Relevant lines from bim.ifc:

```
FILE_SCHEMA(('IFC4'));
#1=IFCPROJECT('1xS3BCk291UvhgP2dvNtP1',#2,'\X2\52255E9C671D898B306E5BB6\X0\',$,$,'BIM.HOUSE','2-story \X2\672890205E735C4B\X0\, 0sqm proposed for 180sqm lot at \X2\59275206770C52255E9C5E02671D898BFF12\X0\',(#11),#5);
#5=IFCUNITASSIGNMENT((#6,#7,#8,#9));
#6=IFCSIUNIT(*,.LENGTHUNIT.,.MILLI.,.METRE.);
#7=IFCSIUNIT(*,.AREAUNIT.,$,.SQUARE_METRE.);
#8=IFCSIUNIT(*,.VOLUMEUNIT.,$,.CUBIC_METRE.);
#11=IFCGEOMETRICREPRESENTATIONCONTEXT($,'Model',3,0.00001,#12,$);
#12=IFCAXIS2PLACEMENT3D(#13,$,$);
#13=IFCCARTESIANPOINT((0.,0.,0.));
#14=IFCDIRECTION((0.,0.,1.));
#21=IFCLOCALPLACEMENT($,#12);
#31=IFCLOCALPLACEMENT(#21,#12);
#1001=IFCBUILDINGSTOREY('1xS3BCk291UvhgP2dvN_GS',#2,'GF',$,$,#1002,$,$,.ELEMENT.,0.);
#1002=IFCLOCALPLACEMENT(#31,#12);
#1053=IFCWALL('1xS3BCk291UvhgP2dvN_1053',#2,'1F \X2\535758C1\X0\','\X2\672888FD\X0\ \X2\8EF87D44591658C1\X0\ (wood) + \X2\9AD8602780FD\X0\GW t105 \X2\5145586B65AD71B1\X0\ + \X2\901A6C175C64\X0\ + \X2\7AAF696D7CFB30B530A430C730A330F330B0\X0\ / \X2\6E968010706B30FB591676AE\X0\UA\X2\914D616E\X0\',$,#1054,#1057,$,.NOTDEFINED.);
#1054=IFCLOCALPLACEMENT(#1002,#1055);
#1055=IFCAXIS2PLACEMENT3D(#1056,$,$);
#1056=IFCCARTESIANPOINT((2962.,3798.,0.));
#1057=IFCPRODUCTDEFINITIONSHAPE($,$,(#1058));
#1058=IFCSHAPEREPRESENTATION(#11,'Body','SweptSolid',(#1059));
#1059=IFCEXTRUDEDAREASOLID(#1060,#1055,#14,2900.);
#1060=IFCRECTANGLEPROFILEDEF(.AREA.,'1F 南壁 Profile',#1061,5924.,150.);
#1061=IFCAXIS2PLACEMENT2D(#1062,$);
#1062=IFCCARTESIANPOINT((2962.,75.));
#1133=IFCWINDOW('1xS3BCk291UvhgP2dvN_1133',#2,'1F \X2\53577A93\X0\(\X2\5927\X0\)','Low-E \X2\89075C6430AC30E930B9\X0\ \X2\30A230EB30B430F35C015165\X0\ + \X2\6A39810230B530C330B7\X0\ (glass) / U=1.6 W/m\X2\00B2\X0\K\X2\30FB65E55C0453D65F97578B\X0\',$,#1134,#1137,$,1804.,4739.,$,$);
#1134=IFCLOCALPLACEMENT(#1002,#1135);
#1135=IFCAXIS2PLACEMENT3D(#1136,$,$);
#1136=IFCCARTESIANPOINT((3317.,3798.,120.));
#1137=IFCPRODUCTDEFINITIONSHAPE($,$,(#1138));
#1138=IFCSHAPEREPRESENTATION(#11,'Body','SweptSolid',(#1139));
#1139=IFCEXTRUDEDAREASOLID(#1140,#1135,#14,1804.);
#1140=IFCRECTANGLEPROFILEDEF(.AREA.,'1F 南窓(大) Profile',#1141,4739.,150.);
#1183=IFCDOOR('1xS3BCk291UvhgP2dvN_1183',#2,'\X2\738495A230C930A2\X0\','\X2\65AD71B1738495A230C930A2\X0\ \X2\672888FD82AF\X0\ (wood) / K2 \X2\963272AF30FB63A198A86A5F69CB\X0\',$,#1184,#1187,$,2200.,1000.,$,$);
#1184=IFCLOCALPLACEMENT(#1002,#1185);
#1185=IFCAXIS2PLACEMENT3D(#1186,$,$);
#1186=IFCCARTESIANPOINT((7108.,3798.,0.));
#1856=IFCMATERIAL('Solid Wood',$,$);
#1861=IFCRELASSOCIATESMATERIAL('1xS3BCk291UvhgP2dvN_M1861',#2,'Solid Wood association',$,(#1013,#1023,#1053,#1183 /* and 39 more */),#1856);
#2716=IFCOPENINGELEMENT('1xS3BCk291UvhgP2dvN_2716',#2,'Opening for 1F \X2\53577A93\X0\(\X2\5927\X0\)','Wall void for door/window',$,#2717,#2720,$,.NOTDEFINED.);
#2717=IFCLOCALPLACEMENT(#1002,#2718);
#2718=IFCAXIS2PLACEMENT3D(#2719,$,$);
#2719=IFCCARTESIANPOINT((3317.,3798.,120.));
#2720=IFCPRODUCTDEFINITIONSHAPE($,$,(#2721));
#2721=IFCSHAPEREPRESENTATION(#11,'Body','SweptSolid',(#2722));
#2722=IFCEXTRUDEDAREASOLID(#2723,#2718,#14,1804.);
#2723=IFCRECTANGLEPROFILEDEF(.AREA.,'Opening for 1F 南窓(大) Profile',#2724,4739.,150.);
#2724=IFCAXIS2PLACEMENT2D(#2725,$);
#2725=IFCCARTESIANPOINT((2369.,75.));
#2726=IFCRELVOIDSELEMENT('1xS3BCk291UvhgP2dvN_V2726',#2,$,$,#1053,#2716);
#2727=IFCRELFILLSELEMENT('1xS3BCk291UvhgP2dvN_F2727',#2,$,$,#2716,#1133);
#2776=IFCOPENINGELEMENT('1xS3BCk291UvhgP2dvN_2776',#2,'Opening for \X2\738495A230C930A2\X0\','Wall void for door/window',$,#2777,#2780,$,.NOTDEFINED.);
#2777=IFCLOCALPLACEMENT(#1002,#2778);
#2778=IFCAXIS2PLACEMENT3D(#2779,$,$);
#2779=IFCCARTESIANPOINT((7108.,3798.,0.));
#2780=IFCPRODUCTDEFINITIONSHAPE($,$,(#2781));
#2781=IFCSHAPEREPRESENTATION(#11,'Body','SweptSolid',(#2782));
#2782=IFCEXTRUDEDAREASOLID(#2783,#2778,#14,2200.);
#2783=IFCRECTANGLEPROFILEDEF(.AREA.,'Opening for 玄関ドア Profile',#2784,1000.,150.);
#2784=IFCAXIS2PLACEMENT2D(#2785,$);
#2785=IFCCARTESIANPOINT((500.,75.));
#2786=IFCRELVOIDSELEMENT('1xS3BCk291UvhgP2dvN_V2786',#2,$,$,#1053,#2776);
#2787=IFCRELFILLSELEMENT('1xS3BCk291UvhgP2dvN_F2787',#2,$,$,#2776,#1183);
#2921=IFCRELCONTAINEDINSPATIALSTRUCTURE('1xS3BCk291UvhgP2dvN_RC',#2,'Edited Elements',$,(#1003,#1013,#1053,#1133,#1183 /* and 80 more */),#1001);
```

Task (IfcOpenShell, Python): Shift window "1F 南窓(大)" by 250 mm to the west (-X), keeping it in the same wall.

```python
import ifcopenshell
import ifcopenshell.api.geometry
import ifcopenshell.util.placement

model = ifcopenshell.open("bim.ifc")

window = model.by_guid("1xS3BCk291UvhgP2dvN_1133")
opening = window.FillsVoids[0].RelatingOpeningElement
wall = opening.VoidsElements[0].RelatingBuildingElement

wall_matrix = ifcopenshell.util.placement.get_local_placement(wall.ObjectPlacement)
shift = wall_matrix[:3, 0] * -250.0
before = ifcopenshell.util.placement.get_local_placement(window.ObjectPlacement)[:3, 3].copy()

# The window is not placed relative to its opening, so move both.
for product in (opening, window):
    matrix = ifcopenshell.util.placement.get_local_placement(product.ObjectPlacement)
    matrix[:3, 3] += shift
    ifcopenshell.api.geometry.edit_object_placement(model, product=product, matrix=matrix, is_si=False)

after = ifcopenshell.util.placement.get_local_placement(window.ObjectPlacement)[:3, 3]
print("window moved by", (after - before).round(3) + 0.0)

model.write("bim-out.ifc")
```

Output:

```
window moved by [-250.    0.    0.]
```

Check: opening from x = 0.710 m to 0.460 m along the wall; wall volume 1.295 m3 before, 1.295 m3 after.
